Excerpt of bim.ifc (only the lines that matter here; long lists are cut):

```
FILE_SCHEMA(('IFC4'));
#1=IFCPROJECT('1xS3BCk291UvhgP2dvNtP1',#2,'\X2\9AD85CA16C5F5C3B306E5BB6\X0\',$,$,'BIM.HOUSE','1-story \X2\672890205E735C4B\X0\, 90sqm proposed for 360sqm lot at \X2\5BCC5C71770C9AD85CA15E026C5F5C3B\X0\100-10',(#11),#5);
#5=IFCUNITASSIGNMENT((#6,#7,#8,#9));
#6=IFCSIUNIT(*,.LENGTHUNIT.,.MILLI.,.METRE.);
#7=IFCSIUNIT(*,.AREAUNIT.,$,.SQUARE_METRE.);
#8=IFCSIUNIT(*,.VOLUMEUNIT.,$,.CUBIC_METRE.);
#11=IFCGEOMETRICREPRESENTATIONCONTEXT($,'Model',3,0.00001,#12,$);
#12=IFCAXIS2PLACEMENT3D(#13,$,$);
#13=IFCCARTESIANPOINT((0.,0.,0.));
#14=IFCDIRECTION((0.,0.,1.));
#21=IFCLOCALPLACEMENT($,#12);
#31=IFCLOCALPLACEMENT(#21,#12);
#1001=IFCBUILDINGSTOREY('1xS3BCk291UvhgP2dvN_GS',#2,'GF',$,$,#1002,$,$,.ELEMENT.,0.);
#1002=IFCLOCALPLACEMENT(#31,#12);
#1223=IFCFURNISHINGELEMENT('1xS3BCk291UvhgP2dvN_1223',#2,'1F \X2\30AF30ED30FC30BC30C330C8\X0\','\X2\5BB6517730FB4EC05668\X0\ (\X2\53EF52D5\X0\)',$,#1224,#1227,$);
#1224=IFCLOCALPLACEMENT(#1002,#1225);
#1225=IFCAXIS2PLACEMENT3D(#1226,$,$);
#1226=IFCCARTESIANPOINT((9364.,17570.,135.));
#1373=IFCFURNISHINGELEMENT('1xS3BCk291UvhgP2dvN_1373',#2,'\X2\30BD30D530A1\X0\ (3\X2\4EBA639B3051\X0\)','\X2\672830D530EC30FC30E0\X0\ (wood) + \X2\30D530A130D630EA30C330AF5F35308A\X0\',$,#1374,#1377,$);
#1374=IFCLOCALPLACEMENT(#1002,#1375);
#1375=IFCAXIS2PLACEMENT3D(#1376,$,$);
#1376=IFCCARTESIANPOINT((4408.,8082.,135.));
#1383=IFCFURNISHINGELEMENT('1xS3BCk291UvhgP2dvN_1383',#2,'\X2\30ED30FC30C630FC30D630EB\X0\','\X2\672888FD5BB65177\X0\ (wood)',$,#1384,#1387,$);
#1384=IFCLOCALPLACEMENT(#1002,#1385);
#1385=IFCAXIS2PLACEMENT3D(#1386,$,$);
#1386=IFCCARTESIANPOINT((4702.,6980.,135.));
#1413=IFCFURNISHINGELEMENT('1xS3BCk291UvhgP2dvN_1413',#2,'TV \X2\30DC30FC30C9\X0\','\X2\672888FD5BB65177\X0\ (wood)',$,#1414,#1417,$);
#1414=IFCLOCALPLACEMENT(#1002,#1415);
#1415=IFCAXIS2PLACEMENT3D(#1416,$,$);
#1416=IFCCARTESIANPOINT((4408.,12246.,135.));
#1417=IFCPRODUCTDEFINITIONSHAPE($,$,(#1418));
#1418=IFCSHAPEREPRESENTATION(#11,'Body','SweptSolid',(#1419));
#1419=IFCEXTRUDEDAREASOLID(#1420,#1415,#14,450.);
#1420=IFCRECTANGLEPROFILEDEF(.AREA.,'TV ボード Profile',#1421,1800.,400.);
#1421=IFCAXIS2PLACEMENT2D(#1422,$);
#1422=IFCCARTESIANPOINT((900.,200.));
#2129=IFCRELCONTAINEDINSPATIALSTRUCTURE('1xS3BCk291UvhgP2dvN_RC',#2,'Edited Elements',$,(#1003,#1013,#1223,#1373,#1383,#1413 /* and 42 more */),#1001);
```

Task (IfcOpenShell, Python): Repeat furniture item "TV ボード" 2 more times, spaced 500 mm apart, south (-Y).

```python
import numpy as np
import ifcopenshell
import ifcopenshell.api.geometry
import ifcopenshell.api.root
import ifcopenshell.util.element
import ifcopenshell.util.placement
import ifcopenshell.util.unit

model = ifcopenshell.open("bim.ifc")
unit_scale = ifcopenshell.util.unit.calculate_unit_scale(model)


def reuse_history(source, copy):
    """copy_class also copies each property set's owner history, people and application; keep the originals."""
    for rel in copy.IsDefinedBy:
        if rel.is_a("IfcRelDefinesByProperties") and (history := rel.RelatingPropertyDefinition.OwnerHistory):
            rel.RelatingPropertyDefinition.OwnerHistory = source.OwnerHistory
            ifcopenshell.util.element.remove_deep2(model, history)


source = model.by_id(1413)
base = ifcopenshell.util.placement.get_local_placement(source.ObjectPlacement)
step = np.array([0.0, -1.0, 0.0]) * 0.5 / unit_scale

for i in range(1, 3):
    copy = ifcopenshell.api.root.copy_class(model, product=source)
    copy.Representation = ifcopenshell.util.element.copy_deep(
        model, source.Representation, exclude=["IfcGeometricRepresentationContext", "IfcRepresentationMap"]
    )
    reuse_history(source, copy)
    matrix = base.copy()
    matrix[:3, 3] += i * step
    print("added at", matrix[:3, 3].round(3) + 0.0)
    ifcopenshell.api.geometry.edit_object_placement(model, product=copy, matrix=matrix, is_si=False)

model.write("bim_edited.ifc")
```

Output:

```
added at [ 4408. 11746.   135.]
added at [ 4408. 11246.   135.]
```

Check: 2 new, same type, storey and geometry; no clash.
